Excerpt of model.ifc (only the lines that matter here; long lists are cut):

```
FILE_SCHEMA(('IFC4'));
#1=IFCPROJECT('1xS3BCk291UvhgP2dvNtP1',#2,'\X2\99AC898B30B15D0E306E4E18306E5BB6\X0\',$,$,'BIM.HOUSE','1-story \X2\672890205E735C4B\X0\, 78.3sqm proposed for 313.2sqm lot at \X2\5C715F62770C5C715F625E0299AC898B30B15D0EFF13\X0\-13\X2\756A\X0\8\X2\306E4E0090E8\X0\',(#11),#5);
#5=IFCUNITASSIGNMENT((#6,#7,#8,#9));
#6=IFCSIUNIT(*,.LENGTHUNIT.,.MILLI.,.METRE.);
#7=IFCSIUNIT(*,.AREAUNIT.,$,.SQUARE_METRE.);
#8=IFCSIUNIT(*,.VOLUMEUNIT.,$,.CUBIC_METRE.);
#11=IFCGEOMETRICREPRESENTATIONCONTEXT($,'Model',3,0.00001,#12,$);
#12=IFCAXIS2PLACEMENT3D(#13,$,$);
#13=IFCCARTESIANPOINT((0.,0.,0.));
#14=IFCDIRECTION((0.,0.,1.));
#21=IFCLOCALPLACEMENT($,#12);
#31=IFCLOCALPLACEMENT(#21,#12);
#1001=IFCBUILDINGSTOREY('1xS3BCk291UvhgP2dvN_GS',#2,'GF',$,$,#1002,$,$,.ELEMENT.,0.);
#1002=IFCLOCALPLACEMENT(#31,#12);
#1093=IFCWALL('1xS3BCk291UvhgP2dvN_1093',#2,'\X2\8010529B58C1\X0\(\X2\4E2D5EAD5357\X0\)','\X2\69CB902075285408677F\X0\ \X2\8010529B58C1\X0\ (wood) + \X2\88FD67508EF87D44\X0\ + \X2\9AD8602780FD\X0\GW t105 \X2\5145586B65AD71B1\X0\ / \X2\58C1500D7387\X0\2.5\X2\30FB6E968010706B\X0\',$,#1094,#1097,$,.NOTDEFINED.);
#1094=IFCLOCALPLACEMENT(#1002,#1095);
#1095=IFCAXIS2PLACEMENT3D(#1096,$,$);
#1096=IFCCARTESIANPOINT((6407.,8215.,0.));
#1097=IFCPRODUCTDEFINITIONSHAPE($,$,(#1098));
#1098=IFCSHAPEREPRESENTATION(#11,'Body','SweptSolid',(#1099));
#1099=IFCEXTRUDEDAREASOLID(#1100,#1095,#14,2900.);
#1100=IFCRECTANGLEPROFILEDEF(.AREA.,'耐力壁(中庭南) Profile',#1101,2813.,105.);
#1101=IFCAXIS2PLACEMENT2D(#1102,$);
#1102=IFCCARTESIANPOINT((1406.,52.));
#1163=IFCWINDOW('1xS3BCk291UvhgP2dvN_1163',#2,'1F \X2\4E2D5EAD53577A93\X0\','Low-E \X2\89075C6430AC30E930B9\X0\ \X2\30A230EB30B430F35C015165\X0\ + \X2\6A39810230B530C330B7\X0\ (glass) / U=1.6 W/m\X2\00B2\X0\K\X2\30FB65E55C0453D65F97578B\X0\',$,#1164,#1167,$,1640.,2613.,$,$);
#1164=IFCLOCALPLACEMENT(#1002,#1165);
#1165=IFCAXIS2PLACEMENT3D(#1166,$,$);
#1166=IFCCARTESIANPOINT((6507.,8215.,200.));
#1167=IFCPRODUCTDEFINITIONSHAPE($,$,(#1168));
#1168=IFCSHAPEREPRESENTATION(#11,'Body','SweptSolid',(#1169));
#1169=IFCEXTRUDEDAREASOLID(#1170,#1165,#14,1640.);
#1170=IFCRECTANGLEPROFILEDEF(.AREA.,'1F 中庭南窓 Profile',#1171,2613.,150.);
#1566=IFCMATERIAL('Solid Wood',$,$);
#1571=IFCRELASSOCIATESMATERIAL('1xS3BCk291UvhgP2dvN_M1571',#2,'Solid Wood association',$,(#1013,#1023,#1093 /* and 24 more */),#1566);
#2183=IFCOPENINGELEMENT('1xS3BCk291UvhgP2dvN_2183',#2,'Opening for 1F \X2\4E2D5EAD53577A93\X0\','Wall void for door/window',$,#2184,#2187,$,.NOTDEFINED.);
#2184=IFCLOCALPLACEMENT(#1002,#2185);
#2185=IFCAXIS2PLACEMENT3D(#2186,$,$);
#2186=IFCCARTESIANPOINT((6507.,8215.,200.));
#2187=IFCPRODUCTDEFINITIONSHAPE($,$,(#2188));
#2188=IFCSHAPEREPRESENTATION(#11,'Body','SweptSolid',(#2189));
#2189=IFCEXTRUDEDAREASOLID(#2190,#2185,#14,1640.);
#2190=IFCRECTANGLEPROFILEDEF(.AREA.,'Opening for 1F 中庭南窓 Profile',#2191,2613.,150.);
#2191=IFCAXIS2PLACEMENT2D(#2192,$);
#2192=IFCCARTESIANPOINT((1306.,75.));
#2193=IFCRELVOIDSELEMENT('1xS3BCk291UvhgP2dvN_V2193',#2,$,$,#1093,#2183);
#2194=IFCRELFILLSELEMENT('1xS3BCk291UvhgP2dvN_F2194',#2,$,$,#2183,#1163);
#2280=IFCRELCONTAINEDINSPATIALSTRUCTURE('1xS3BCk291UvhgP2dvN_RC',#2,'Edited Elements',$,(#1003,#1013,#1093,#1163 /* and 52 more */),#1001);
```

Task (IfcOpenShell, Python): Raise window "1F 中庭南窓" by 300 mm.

```python
import numpy as np
import ifcopenshell
import ifcopenshell.api.geometry
import ifcopenshell.util.placement
import ifcopenshell.util.unit

model = ifcopenshell.open("model.ifc")
unit_scale = ifcopenshell.util.unit.calculate_unit_scale(model)

window = model.by_id(1163)
opening = window.FillsVoids[0].RelatingOpeningElement
dz = 300.0

shift = np.array([0.0, 0.0, dz])
# The window is not placed relative to its opening, so move both.
for product in (opening, window):
    matrix = ifcopenshell.util.placement.get_local_placement(product.ObjectPlacement)
    matrix[:3, 3] += shift
    ifcopenshell.api.geometry.edit_object_placement(model, product=product, matrix=matrix, is_si=False)

print(f"moved by {dz * unit_scale:+.3f} m")

model.write("model_v2.ifc")
```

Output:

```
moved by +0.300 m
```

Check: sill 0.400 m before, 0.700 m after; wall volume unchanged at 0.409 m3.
